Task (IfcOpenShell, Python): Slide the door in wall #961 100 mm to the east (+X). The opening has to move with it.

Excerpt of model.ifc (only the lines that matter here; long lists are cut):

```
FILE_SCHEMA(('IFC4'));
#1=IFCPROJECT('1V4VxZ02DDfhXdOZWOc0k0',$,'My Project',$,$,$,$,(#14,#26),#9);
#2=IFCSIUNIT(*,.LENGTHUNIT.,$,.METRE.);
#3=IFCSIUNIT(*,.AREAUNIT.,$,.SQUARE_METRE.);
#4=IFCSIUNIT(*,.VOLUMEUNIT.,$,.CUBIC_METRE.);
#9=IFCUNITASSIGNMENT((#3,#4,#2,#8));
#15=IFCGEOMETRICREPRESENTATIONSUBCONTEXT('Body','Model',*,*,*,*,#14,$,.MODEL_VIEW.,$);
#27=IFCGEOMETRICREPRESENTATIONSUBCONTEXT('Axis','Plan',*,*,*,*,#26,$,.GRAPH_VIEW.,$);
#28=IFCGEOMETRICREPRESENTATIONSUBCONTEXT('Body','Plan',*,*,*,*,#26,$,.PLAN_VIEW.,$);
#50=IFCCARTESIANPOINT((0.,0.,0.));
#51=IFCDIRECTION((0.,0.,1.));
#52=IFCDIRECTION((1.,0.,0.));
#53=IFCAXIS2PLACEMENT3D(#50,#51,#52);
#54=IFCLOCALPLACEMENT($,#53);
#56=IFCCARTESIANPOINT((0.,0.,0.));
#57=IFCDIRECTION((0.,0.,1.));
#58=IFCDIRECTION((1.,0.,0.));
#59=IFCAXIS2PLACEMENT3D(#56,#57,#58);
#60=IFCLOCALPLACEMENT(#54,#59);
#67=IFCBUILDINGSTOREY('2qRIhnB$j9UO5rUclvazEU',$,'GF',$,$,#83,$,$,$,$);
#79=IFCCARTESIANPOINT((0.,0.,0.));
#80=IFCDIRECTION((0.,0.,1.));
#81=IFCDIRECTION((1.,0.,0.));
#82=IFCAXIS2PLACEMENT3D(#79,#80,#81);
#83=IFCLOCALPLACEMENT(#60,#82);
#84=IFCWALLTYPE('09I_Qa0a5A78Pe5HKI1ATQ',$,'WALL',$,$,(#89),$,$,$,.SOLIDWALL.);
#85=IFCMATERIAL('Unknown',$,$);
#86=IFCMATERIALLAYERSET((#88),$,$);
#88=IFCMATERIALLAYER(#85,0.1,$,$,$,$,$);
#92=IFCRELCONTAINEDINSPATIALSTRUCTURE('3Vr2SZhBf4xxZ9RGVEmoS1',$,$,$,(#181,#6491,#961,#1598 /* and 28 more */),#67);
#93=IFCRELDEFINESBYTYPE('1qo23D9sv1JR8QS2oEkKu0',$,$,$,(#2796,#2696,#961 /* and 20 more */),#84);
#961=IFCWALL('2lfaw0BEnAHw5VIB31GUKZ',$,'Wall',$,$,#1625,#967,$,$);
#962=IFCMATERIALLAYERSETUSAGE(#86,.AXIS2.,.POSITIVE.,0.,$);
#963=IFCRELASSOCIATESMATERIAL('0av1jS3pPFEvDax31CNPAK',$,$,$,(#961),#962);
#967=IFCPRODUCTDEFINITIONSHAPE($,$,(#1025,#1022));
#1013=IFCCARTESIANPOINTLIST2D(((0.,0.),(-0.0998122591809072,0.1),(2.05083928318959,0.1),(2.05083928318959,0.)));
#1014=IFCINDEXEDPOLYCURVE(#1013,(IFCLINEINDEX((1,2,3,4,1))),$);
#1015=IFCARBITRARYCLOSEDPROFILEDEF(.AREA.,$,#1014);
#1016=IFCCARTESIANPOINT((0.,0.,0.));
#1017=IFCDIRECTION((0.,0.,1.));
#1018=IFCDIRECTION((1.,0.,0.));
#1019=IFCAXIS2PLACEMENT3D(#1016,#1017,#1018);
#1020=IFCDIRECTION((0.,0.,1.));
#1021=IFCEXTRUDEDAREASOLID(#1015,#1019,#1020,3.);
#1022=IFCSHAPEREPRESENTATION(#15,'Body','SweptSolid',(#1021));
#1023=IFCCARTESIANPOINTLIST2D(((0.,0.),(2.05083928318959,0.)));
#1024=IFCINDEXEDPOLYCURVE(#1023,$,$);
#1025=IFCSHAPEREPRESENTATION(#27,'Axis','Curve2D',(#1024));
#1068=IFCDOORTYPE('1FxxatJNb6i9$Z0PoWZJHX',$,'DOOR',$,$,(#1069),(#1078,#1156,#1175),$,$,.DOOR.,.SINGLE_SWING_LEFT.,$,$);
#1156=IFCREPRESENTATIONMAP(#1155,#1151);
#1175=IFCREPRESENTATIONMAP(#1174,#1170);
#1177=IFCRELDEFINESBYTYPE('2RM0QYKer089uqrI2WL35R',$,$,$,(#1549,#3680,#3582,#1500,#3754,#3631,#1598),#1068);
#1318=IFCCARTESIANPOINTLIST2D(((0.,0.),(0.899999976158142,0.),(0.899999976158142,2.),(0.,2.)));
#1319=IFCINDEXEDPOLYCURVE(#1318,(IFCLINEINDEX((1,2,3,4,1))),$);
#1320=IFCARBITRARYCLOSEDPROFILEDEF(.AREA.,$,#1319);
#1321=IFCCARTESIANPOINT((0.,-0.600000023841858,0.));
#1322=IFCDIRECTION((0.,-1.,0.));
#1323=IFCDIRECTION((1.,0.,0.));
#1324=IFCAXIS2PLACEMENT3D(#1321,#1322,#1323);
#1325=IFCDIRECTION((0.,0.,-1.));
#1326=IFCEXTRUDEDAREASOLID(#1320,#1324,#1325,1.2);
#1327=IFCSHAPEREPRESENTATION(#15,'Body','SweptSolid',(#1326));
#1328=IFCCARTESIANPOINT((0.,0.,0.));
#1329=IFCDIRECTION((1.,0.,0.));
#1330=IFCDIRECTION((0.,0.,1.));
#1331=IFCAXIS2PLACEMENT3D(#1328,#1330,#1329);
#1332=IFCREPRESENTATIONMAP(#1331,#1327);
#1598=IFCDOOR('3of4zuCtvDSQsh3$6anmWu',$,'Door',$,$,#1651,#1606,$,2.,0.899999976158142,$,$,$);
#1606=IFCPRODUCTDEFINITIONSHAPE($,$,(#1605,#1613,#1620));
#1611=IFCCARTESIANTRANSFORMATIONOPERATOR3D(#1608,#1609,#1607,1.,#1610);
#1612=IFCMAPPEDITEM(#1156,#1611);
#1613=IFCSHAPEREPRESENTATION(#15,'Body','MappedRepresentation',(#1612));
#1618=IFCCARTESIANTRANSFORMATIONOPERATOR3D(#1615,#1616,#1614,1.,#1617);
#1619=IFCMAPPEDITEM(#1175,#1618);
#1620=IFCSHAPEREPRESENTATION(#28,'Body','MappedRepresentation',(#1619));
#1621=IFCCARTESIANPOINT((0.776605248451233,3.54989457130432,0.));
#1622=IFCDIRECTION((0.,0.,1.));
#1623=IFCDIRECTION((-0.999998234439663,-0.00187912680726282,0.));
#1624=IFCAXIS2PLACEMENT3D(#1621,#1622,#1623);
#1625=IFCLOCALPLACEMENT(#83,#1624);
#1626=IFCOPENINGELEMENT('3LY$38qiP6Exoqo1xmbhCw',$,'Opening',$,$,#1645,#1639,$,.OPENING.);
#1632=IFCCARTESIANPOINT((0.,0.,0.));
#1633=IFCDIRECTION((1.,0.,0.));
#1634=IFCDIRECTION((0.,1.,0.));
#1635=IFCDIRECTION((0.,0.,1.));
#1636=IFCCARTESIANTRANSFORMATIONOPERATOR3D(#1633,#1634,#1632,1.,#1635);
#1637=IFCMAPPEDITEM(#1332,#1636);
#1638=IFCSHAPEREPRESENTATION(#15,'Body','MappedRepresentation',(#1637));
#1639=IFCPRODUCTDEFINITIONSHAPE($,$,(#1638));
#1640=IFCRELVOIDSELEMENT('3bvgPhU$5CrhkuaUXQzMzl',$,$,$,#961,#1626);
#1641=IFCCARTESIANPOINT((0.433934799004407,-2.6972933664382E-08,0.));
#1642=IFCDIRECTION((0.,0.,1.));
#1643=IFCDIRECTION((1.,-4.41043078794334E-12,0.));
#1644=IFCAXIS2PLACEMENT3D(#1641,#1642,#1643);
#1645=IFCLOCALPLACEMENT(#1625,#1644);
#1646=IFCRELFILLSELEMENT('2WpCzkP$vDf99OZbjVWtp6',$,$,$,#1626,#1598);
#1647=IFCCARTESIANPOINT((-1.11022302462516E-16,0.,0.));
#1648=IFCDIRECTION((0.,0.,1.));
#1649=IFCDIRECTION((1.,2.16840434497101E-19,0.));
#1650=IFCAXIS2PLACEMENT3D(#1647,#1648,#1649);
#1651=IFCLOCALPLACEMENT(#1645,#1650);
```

```python
import ifcopenshell
import ifcopenshell.api.geometry
import ifcopenshell.util.placement
import ifcopenshell.util.unit

model = ifcopenshell.open("model.ifc")
unit_scale = ifcopenshell.util.unit.calculate_unit_scale(model)

door = model.by_guid("3of4zuCtvDSQsh3$6anmWu")
opening = door.FillsVoids[0].RelatingOpeningElement
wall = opening.VoidsElements[0].RelatingBuildingElement

wall_matrix = ifcopenshell.util.placement.get_local_placement(wall.ObjectPlacement)
shift = wall_matrix[:3, 0] * -0.1 / unit_scale
before = ifcopenshell.util.placement.get_local_placement(door.ObjectPlacement)[:3, 3].copy()

# The door is placed relative to its opening, so it follows when the opening moves.
matrix = ifcopenshell.util.placement.get_local_placement(opening.ObjectPlacement)
matrix[:3, 3] += shift
ifcopenshell.api.geometry.edit_object_placement(
    model, product=opening, matrix=matrix, is_si=False, should_transform_children=True
)

after = ifcopenshell.util.placement.get_local_placement(door.ObjectPlacement)[:3, 3]
print("door moved by", (after - before).round(3) + 0.0)

model.write("model-out.ifc")
```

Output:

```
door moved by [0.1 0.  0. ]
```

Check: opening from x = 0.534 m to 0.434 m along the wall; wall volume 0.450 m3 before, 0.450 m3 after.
